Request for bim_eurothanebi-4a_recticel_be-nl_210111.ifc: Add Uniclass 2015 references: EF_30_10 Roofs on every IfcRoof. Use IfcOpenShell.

First a look at what the model holds.

```python
import ifcopenshell

model = ifcopenshell.open("bim_eurothanebi-4a_recticel_be-nl_210111.ifc")
print(model.schema)
print("classifications:", [c.Name for c in model.by_type("IfcClassification")])
for ifc_class in ("IfcDoor", "IfcRoof", "IfcStair", "IfcWall", "IfcWindow"):
    print(ifc_class, len(model.by_type(ifc_class)))
```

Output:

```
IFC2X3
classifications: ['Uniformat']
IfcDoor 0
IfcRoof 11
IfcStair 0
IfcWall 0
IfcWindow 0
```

```python
import ifcopenshell
import ifcopenshell.api.classification

model = ifcopenshell.open("bim_eurothanebi-4a_recticel_be-nl_210111.ifc")

# IFC2X3 requires Source and Edition and has no link from the project to the system.
system = model.create_entity("IfcClassification", Source="NBS", Edition="2015", Name="Uniclass 2015")

codes = {
    "IfcRoof": ("EF_30_10", "Roofs"),
}
for ifc_class, (code, name) in codes.items():
    products = model.by_type(ifc_class)
    ifcopenshell.api.classification.add_reference(
        model, products=products, classification=system, identification=code, name=name
    )
    print(code, len(products))

model.write("bim_eurothanebi-4a_recticel_be-nl_210111_v2.ifc")
```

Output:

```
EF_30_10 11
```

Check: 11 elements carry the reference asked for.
